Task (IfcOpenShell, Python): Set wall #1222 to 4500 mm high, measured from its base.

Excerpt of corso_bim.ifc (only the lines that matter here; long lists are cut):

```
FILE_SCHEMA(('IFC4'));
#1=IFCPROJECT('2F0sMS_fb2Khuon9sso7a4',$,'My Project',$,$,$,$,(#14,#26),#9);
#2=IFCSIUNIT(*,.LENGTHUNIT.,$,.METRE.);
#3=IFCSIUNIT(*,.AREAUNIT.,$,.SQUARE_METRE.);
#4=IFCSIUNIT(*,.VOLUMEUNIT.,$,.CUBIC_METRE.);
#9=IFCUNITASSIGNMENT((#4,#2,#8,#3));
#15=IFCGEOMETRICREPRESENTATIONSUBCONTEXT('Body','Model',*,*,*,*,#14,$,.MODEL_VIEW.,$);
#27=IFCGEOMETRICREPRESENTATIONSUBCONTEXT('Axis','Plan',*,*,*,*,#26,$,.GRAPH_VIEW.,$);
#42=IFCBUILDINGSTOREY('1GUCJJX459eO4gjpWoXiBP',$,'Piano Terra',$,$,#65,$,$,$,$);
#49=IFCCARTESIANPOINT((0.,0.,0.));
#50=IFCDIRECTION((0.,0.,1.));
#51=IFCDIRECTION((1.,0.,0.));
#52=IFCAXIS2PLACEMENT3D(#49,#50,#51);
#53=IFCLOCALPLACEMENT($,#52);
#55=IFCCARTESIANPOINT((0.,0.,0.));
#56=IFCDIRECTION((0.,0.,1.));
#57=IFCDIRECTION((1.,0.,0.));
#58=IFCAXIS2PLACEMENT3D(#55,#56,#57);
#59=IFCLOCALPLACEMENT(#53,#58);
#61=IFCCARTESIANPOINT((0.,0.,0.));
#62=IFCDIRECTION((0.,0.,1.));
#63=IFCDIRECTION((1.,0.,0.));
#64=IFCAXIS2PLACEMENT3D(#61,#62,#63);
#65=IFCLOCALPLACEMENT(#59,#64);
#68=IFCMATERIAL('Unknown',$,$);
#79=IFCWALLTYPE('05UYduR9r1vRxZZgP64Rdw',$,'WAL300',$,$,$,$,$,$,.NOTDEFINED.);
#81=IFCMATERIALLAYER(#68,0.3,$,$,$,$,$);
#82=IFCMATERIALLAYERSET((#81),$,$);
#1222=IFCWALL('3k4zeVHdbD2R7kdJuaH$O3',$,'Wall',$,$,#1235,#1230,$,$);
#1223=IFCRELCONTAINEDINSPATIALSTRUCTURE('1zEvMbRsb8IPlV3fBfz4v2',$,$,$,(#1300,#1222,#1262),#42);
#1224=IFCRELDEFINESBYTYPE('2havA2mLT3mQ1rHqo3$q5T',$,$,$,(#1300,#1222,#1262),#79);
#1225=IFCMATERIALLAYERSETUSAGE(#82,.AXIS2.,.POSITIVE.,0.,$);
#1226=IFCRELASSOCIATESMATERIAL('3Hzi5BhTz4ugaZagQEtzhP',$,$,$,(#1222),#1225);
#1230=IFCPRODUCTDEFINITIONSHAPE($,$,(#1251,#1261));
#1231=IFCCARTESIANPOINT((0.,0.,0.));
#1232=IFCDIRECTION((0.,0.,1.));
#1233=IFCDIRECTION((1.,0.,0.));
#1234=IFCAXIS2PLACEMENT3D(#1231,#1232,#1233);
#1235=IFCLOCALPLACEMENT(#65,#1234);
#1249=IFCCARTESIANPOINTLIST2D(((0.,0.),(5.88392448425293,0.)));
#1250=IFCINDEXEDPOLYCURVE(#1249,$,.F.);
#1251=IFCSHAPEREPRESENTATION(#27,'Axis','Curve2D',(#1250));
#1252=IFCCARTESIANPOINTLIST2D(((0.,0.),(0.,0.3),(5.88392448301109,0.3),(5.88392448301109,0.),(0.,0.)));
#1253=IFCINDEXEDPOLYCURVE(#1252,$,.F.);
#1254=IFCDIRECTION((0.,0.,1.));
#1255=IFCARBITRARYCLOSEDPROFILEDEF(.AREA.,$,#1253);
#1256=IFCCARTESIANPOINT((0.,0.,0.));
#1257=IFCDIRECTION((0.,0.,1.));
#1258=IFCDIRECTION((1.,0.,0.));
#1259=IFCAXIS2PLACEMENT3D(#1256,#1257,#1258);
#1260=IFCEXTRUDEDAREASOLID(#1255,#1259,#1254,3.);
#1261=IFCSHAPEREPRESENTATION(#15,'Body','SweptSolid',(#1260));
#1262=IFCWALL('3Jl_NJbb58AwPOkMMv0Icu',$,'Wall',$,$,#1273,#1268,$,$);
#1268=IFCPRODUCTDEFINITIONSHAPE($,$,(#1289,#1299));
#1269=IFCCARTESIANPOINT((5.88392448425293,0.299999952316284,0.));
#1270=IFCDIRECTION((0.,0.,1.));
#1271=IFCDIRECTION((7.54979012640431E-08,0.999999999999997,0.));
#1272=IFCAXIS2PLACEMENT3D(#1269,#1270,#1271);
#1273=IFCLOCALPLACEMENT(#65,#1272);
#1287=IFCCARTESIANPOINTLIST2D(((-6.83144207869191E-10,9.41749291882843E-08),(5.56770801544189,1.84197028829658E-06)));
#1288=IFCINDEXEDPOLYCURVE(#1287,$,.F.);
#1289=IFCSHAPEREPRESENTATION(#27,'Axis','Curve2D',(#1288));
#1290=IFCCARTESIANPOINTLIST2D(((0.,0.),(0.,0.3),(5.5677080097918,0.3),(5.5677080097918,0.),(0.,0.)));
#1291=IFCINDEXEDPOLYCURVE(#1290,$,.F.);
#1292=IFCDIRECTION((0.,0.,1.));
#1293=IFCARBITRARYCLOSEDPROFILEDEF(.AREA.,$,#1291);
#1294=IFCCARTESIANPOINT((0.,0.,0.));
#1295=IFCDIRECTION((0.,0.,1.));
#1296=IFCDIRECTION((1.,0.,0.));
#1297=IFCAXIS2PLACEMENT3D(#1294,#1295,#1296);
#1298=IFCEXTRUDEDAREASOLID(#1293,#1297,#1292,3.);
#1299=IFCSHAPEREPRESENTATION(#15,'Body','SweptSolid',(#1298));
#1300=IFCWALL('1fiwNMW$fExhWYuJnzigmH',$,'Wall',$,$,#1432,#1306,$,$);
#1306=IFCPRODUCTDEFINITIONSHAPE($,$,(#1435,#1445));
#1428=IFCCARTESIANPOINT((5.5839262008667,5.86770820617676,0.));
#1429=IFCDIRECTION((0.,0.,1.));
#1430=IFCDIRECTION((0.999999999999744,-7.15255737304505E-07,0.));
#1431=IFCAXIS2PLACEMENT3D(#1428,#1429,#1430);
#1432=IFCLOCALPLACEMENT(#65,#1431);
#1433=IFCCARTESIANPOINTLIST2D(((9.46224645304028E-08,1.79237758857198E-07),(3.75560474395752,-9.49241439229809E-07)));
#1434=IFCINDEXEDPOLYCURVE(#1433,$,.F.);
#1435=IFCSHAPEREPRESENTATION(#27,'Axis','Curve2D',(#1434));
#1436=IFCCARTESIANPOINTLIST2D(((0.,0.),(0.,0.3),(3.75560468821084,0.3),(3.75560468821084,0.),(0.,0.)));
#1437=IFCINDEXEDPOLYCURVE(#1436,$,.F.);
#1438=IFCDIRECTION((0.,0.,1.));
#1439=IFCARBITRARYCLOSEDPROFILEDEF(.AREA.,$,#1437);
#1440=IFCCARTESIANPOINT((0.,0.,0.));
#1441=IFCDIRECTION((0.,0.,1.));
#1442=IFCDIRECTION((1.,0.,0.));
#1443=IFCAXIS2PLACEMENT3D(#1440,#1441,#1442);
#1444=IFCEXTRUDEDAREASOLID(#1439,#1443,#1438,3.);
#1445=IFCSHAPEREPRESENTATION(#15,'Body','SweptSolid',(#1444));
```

```python
import ifcopenshell
import ifcopenshell.geom
import ifcopenshell.util.representation
import ifcopenshell.util.shape
import ifcopenshell.util.unit

model = ifcopenshell.open("corso_bim.ifc")
unit_scale = ifcopenshell.util.unit.calculate_unit_scale(model)
settings = ifcopenshell.geom.settings()


def volume(element):
    """Net volume in cubic metres, openings subtracted."""
    shape = ifcopenshell.geom.create_shape(settings, element)
    return ifcopenshell.util.shape.get_volume(shape.geometry)


wall = model.by_id(1222)
before = volume(wall)

body = ifcopenshell.util.representation.get_representation(wall, "Model", "Body")
solid = body.Items[0]
old_height = solid.Depth
solid.Depth = 4.5 / unit_scale
after = volume(wall)

print(f"height {old_height:g} -> {solid.Depth:g}, volume {before:.3f} -> {after:.3f} m3")

model.write("corso_bim_v2.ifc")
```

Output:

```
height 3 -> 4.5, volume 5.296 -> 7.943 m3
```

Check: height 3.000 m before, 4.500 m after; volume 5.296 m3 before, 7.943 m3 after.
